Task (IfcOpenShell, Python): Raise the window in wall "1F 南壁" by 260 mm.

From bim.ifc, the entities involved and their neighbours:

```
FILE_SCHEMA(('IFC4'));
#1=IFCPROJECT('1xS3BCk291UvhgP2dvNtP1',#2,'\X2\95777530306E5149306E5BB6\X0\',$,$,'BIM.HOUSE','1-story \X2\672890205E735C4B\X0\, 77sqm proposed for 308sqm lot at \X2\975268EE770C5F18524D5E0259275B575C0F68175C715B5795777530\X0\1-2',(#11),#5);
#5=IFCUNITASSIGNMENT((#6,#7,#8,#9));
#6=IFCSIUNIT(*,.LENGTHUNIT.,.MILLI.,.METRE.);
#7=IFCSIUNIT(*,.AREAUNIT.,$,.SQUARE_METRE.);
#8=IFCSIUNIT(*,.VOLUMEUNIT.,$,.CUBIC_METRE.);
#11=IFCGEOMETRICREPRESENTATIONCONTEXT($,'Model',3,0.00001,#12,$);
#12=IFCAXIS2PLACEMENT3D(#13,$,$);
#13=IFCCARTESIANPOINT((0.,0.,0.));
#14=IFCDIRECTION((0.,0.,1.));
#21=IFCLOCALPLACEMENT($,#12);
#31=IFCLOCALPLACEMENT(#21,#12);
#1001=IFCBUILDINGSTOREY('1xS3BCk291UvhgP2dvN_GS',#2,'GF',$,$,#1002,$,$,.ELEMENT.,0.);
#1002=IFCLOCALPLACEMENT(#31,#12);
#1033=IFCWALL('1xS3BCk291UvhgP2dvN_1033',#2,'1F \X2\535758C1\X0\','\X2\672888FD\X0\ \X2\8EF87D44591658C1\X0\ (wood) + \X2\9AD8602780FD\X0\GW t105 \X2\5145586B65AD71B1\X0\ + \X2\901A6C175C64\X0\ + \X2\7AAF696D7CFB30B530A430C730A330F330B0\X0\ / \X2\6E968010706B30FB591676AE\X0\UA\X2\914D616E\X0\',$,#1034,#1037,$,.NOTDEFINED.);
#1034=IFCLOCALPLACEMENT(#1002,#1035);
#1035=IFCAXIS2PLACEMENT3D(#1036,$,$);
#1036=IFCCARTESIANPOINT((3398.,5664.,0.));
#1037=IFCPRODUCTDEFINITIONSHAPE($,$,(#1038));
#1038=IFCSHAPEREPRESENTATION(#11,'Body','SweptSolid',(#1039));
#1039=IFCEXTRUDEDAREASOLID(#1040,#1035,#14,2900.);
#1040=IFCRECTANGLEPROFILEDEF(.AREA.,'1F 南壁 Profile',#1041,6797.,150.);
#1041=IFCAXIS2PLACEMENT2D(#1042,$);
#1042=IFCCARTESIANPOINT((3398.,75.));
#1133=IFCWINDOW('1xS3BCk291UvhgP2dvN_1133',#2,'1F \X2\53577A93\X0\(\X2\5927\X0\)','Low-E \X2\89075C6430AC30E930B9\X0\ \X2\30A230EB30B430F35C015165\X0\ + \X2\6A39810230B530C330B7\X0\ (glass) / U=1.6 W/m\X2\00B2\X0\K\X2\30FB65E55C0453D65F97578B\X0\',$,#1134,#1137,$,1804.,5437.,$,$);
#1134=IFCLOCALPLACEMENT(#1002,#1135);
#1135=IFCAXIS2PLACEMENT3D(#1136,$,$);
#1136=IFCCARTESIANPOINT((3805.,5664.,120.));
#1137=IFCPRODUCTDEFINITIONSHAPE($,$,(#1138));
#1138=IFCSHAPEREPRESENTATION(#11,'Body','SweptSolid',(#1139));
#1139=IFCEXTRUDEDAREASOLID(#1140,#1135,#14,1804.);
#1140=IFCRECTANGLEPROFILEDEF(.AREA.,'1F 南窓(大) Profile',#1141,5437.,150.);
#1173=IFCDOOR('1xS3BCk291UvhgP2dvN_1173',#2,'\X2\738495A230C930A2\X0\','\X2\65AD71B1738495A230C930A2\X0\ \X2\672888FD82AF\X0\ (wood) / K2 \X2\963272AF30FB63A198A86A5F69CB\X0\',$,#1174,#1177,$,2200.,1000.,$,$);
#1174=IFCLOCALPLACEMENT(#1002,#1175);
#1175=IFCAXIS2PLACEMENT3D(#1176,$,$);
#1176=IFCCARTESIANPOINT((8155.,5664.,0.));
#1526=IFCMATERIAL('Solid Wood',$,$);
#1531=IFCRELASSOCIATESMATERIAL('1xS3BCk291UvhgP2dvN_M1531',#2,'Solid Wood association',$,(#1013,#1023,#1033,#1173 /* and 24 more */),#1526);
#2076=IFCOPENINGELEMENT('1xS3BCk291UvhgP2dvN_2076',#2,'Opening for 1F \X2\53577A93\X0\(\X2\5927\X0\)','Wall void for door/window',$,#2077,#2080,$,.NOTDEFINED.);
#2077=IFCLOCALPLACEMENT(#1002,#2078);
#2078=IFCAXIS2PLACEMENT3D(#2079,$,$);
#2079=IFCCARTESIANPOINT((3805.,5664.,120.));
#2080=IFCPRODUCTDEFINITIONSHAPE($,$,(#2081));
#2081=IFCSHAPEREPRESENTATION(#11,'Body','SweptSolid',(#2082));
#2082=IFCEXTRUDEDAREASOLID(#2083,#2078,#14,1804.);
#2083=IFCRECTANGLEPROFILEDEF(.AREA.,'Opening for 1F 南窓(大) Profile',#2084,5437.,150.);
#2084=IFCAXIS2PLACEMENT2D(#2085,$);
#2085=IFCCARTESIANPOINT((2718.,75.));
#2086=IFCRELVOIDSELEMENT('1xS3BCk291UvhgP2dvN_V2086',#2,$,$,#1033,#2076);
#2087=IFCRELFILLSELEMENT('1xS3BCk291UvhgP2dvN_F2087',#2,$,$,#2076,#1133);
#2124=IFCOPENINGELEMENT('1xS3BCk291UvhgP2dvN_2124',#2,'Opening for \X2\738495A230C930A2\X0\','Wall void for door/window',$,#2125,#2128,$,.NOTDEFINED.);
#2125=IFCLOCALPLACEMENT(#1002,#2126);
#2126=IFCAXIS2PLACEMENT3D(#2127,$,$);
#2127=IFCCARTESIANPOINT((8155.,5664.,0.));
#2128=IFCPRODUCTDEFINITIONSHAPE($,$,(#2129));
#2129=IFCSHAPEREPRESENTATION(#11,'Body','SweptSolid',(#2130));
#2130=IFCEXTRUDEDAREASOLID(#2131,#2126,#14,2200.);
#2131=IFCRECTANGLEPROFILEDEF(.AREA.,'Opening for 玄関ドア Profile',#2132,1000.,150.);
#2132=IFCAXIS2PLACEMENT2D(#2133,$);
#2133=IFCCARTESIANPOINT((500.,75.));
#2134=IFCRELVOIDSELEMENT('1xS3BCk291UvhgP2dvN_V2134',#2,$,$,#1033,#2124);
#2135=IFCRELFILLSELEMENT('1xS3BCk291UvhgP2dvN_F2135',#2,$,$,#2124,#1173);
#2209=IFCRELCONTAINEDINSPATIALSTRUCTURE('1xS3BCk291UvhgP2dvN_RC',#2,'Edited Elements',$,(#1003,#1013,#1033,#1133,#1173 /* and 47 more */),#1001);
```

```python
import numpy as np
import ifcopenshell
import ifcopenshell.api.geometry
import ifcopenshell.util.placement
import ifcopenshell.util.unit

model = ifcopenshell.open("bim.ifc")
unit_scale = ifcopenshell.util.unit.calculate_unit_scale(model)

window = model.by_guid("1xS3BCk291UvhgP2dvN_1133")
opening = window.FillsVoids[0].RelatingOpeningElement
dz = 260.0

shift = np.array([0.0, 0.0, dz])
# The window is not placed relative to its opening, so move both.
for product in (opening, window):
    matrix = ifcopenshell.util.placement.get_local_placement(product.ObjectPlacement)
    matrix[:3, 3] += shift
    ifcopenshell.api.geometry.edit_object_placement(model, product=product, matrix=matrix, is_si=False)

print(f"moved by {dz * unit_scale:+.3f} m")

model.write("bim_updated.ifc")
```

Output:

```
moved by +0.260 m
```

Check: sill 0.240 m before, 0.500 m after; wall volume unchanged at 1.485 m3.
